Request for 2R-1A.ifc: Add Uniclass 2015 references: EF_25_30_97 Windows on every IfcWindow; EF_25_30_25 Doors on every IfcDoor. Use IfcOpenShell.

First a look at what the model holds.

```python
import ifcopenshell

model = ifcopenshell.open("2R-1A.ifc")
print(model.schema)
print("classifications:", [c.Name for c in model.by_type("IfcClassification")])
for ifc_class in ("IfcDoor", "IfcRoof", "IfcStair", "IfcWall", "IfcWindow"):
    print(ifc_class, len(model.by_type(ifc_class)))
```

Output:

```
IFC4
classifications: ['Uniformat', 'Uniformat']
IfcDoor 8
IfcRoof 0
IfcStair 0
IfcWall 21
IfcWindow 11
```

```python
import ifcopenshell
import ifcopenshell.api.classification

model = ifcopenshell.open("2R-1A.ifc")

system = ifcopenshell.api.classification.add_classification(model, classification="Uniclass 2015")

codes = {
    "IfcWindow": ("EF_25_30_97", "Windows"),
    "IfcDoor": ("EF_25_30_25", "Doors"),
}
for ifc_class, (code, name) in codes.items():
    products = model.by_type(ifc_class)
    ifcopenshell.api.classification.add_reference(
        model, products=products, classification=system, identification=code, name=name
    )
    print(code, len(products))

model.write("2R-1A_updated.ifc")
```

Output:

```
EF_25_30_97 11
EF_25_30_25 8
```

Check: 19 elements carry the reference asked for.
